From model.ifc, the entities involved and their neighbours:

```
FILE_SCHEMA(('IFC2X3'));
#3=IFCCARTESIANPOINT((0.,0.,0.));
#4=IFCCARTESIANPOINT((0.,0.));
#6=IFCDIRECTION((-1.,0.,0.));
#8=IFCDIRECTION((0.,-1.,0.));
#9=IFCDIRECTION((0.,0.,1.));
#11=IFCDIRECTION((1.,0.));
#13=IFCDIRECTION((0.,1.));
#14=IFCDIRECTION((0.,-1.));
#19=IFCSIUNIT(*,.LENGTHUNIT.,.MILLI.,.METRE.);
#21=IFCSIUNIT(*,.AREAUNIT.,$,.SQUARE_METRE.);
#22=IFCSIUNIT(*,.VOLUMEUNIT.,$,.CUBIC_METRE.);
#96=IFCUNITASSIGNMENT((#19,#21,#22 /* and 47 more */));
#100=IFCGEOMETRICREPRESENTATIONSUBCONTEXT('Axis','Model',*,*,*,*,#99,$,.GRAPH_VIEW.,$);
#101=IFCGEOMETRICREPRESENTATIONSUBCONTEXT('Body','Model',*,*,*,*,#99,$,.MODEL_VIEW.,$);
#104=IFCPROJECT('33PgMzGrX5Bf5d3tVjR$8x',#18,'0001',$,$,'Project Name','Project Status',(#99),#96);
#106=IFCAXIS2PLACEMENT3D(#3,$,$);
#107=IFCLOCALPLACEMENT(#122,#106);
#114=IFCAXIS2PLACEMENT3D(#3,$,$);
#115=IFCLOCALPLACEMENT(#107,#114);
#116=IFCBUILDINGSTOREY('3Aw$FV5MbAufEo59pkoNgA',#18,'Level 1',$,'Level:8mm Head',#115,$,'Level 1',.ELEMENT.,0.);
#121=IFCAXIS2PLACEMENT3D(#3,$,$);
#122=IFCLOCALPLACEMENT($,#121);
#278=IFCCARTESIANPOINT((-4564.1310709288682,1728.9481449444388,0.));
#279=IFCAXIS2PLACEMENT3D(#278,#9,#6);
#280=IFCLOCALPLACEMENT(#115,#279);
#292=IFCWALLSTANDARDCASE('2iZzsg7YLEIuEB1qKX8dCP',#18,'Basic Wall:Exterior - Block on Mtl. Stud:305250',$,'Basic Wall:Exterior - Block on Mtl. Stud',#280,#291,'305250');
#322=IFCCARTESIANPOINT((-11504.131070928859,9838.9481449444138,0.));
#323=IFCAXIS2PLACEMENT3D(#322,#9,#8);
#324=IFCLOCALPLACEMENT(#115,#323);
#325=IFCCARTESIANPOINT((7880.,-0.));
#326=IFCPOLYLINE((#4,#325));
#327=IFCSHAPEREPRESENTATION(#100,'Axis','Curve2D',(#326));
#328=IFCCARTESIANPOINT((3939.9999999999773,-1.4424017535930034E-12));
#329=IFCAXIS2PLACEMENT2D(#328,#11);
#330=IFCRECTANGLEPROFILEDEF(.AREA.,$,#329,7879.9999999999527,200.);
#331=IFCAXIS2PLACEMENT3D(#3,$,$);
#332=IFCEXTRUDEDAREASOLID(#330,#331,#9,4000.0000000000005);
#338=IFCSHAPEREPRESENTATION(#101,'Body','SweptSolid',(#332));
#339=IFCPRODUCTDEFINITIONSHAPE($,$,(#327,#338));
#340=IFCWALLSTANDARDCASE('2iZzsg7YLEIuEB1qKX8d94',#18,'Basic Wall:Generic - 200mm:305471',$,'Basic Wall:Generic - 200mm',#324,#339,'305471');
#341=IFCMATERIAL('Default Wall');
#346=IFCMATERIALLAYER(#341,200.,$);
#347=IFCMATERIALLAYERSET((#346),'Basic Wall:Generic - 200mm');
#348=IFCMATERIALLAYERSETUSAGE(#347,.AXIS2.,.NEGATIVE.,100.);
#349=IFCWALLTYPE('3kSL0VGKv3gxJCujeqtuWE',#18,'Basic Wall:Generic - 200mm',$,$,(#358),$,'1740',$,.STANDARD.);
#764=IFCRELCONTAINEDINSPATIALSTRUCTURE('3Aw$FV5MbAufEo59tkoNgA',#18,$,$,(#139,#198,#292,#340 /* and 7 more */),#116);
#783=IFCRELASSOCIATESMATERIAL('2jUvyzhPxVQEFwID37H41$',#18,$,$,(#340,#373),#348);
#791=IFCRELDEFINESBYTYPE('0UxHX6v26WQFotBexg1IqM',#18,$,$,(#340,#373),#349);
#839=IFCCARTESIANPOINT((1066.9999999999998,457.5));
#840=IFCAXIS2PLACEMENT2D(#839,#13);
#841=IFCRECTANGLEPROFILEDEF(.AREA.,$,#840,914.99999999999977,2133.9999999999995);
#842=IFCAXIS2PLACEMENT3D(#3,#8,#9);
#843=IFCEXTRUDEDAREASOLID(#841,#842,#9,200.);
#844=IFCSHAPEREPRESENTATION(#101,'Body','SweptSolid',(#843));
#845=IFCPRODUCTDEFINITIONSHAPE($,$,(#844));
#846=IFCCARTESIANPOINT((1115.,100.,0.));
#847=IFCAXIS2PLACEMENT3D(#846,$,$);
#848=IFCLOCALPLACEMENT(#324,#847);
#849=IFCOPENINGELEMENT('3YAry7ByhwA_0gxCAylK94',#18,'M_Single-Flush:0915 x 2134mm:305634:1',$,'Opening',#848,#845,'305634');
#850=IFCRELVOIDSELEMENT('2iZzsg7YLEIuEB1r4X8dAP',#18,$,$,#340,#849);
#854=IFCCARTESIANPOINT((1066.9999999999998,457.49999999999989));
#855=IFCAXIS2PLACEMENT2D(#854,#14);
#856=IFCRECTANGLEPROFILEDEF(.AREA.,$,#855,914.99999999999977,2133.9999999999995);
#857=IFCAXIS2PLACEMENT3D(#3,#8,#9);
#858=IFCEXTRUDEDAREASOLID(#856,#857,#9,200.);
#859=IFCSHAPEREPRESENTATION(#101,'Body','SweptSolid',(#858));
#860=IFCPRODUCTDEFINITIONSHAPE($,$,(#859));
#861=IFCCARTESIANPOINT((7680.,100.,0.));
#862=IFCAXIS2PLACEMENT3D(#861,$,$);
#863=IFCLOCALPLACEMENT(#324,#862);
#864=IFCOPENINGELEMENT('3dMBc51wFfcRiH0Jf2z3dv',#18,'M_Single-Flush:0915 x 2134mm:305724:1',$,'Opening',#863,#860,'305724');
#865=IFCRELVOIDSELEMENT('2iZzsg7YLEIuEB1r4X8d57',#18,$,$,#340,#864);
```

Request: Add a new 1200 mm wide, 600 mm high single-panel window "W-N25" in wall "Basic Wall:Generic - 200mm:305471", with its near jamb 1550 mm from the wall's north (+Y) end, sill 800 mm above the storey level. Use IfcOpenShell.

```python
import numpy as np
import ifcopenshell
import ifcopenshell.api.feature
import ifcopenshell.api.geometry
import ifcopenshell.api.root
import ifcopenshell.api.spatial
import ifcopenshell.api.type
import ifcopenshell.geom
import ifcopenshell.util.element
import ifcopenshell.util.placement
import ifcopenshell.util.representation
import ifcopenshell.util.shape
import ifcopenshell.util.unit

model = ifcopenshell.open("model.ifc")
unit_scale = ifcopenshell.util.unit.calculate_unit_scale(model)
settings = ifcopenshell.geom.settings()


def volume(element):
    """Net volume in cubic metres, openings subtracted."""
    shape = ifcopenshell.geom.create_shape(settings, element)
    return ifcopenshell.util.shape.get_volume(shape.geometry)


wall = model.by_guid("2iZzsg7YLEIuEB1qKX8d94")
storey = ifcopenshell.util.element.get_container(wall, ifc_class="IfcBuildingStorey")
context = ifcopenshell.util.representation.get_context(model, "Model", "Body", "MODEL_VIEW")
before = volume(wall)

width, height, from_end, sill = 1.2, 0.6, 1.55, 0.8  # metres

# The wall runs along its own X axis, and the end named is its -X end.
wall_shape = ifcopenshell.geom.create_shape(settings, wall)
x, y, z = ifcopenshell.util.shape.get_vertices(wall_shape.geometry).T
start = x.min() + from_end
face, thickness = float(y.min()), float(y.max() - y.min())
wall_matrix = ifcopenshell.util.placement.get_local_placement(wall.ObjectPlacement)
level = ifcopenshell.util.placement.get_local_placement(storey.ObjectPlacement)[2, 3]


def in_wall(x, y):
    """Placement at x, y metres in the wall's axes, at sill height."""
    matrix = wall_matrix.copy()
    matrix[:, 3] = wall_matrix @ np.array([x / unit_scale, y / unit_scale, 0.0, 1.0])
    matrix[2, 3] = level + sill / unit_scale
    return matrix


# Opening: a box that overshoots both wall faces by 50 mm.
opening = ifcopenshell.api.root.create_entity(model, ifc_class="IfcOpeningElement")
box = ifcopenshell.api.geometry.add_wall_representation(
    model, context=context, length=width, height=height, thickness=thickness + 0.1
)
ifcopenshell.api.geometry.assign_representation(model, product=opening, representation=box)
ifcopenshell.api.geometry.edit_object_placement(model, product=opening, matrix=in_wall(start, face - 0.05), is_si=False)
ifcopenshell.api.feature.add_feature(model, feature=opening, element=wall)

window = ifcopenshell.api.root.create_entity(model, ifc_class="IfcWindow", name="W-N25")
window.OverallWidth, window.OverallHeight = width / unit_scale, height / unit_scale
body = ifcopenshell.api.geometry.add_window_representation(
    model,
    context=context,
    overall_width=window.OverallWidth,
    overall_height=window.OverallHeight,
    partition_type="SINGLE_PANEL",
)
ifcopenshell.api.geometry.assign_representation(model, product=window, representation=body)
ifcopenshell.api.spatial.assign_container(model, products=[window], relating_structure=storey)
fills = ifcopenshell.api.feature.add_filling(model, opening=opening, element=window)
fills.OwnerHistory = window.OwnerHistory  # required in IFC2X3

# IFC2X3 keeps the operation on the window style.
style = ifcopenshell.api.root.create_entity(model, ifc_class="IfcWindowStyle", name="W-N25")
style.OperationType, style.ConstructionType = "SINGLE_PANEL", "NOTDEFINED"
style.ParameterTakesPrecedence = style.Sizeable = False
ifcopenshell.api.type.assign_type(model, related_objects=[window], relating_type=style)

# Centre the window in the wall's thickness.
ifcopenshell.api.geometry.edit_object_placement(model, product=window, matrix=in_wall(start, face), is_si=False)
window_shape = ifcopenshell.geom.create_shape(settings, window)
depth = ifcopenshell.util.shape.get_vertices(window_shape.geometry)[:, 1]
offset = face + thickness / 2 - (depth.min() + depth.max()) / 2
ifcopenshell.api.geometry.edit_object_placement(model, product=window, matrix=in_wall(start, offset), is_si=False)

after = volume(wall)

print(f"wall volume {before:.3f} -> {after:.3f} m3")

model.write("model-out.ifc")
```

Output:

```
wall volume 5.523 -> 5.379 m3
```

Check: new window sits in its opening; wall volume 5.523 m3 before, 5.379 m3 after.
